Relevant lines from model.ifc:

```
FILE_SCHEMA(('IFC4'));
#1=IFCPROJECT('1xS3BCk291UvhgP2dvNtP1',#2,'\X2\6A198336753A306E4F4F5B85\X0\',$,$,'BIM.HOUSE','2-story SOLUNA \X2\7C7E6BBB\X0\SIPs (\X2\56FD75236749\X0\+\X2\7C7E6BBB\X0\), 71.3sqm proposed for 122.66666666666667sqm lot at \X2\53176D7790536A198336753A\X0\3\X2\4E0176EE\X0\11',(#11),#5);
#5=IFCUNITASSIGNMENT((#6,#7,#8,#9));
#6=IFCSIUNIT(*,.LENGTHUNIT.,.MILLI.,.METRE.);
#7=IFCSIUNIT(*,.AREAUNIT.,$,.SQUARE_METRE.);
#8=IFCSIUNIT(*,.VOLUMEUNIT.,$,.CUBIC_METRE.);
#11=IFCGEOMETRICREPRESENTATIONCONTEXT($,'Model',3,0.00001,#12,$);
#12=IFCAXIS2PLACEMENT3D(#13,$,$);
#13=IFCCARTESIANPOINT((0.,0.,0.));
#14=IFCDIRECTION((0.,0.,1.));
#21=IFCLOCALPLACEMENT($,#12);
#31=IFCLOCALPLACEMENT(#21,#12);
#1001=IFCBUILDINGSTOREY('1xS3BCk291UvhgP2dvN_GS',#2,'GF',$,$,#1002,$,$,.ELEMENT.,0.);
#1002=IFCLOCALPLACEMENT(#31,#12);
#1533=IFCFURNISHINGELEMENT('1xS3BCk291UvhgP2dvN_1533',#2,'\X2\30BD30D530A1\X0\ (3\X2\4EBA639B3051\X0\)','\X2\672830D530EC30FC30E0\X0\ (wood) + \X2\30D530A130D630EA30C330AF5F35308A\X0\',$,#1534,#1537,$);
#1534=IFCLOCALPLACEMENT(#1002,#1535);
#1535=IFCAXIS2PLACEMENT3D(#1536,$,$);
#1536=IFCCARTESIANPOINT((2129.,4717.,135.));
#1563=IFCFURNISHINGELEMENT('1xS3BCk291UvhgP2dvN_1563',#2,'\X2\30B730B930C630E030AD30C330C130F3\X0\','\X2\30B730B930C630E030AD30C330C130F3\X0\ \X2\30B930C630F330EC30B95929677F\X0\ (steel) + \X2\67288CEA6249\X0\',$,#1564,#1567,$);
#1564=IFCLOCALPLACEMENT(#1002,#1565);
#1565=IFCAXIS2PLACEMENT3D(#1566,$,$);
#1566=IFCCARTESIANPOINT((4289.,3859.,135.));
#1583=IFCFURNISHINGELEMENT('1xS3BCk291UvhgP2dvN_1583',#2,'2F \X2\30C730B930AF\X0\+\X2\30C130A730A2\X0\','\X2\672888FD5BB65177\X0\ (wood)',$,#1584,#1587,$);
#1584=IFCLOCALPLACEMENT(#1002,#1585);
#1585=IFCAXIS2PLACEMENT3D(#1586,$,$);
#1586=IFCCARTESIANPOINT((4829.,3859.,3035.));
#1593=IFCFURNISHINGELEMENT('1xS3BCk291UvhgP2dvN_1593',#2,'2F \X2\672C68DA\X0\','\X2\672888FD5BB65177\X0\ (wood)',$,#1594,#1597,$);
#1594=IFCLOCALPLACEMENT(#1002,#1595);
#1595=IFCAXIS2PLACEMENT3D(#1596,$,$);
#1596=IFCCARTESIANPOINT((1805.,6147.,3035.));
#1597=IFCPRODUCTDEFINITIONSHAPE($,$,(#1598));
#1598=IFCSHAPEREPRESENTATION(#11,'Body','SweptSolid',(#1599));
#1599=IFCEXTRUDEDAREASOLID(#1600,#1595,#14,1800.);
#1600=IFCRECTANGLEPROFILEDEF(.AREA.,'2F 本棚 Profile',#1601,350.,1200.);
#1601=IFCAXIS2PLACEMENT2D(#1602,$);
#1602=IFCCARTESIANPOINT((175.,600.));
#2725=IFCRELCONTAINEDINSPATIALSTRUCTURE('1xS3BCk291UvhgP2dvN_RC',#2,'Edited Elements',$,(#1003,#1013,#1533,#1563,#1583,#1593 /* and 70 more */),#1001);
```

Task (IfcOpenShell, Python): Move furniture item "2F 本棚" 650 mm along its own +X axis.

```python
import ifcopenshell
import ifcopenshell.api.geometry
import ifcopenshell.util.placement

model = ifcopenshell.open("model.ifc")

item = model.by_guid("1xS3BCk291UvhgP2dvN_1593")
matrix = ifcopenshell.util.placement.get_local_placement(item.ObjectPlacement)
matrix[:3, 3] += matrix[:3, 0] * 650.0
ifcopenshell.api.geometry.edit_object_placement(model, product=item, matrix=matrix, is_si=False)

print(ifcopenshell.util.placement.get_local_placement(item.ObjectPlacement).round(3) + 0.0)

model.write("model_rev.ifc")
```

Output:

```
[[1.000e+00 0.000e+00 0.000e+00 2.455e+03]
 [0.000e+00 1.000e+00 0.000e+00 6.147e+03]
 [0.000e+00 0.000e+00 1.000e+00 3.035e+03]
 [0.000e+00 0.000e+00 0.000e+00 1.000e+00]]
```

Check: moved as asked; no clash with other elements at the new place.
